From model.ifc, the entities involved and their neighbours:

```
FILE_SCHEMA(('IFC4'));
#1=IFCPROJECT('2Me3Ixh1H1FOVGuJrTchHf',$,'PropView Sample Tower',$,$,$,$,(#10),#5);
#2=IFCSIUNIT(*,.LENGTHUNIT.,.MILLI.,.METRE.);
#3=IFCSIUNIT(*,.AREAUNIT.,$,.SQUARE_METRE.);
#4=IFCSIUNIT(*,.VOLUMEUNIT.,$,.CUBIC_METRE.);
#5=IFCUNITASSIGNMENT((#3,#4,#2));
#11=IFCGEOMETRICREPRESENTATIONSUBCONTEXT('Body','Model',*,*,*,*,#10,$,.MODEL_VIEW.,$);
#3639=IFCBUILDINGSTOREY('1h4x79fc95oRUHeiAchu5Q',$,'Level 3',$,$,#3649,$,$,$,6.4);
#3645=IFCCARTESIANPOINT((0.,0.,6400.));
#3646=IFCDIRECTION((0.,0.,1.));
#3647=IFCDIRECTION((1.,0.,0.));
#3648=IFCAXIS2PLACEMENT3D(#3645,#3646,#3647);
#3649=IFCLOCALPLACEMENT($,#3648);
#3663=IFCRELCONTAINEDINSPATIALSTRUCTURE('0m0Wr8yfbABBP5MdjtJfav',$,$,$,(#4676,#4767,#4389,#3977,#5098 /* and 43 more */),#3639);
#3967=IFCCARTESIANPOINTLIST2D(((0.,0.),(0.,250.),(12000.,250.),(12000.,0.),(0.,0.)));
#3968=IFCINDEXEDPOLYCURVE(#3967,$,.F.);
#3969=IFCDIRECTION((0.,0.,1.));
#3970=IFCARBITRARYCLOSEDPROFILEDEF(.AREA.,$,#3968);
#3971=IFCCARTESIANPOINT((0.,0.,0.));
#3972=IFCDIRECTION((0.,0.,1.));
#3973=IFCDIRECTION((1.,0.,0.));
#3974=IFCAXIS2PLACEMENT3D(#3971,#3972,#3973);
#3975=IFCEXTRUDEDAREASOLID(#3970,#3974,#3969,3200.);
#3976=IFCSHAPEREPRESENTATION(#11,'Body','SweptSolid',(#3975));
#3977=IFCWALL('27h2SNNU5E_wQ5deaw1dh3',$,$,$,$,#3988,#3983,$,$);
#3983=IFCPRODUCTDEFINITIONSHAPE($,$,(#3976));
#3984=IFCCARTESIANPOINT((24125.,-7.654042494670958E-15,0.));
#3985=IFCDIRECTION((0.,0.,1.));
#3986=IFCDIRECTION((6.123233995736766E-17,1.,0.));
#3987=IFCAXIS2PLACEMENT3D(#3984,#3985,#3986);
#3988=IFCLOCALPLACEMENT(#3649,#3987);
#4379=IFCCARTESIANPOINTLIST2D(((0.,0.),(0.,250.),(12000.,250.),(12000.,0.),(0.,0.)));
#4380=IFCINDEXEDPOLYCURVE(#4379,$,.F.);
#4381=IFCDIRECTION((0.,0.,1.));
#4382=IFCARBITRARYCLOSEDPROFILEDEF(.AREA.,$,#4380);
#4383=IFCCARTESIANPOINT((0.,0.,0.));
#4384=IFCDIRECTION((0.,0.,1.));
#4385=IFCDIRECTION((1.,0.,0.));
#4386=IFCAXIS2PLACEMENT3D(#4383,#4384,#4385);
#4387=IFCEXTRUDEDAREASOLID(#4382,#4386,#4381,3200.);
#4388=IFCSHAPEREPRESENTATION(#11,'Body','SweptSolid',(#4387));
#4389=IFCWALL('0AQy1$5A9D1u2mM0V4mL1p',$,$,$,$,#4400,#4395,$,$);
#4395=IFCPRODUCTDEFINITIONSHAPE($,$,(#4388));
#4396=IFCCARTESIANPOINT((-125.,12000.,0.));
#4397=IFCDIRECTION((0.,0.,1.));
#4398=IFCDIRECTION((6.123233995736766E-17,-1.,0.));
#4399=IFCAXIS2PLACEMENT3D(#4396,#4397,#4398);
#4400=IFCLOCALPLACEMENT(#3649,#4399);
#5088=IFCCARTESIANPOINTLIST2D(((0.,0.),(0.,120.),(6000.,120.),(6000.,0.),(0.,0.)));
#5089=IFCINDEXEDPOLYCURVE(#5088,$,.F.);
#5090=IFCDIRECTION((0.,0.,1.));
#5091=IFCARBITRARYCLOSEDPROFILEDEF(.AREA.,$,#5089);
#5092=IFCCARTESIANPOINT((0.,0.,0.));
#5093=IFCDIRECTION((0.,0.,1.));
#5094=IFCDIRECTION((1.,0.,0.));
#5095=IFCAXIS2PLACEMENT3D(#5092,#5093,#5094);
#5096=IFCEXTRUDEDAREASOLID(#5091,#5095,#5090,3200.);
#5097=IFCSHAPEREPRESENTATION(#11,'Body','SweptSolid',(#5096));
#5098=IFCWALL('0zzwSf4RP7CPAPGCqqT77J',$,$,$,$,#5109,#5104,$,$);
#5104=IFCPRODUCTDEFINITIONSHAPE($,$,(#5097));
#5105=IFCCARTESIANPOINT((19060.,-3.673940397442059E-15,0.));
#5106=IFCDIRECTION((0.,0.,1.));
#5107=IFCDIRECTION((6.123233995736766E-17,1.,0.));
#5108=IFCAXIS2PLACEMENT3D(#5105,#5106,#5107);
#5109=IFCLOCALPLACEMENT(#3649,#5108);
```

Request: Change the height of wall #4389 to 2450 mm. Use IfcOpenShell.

```python
import ifcopenshell
import ifcopenshell.geom
import ifcopenshell.util.representation
import ifcopenshell.util.shape
import ifcopenshell.util.unit

model = ifcopenshell.open("model.ifc")
unit_scale = ifcopenshell.util.unit.calculate_unit_scale(model)
settings = ifcopenshell.geom.settings()


def volume(element):
    """Net volume in cubic metres, openings subtracted."""
    shape = ifcopenshell.geom.create_shape(settings, element)
    return ifcopenshell.util.shape.get_volume(shape.geometry)


wall = model.by_id(4389)
before = volume(wall)

body = ifcopenshell.util.representation.get_representation(wall, "Model", "Body")
solid = body.Items[0]
old_height = solid.Depth
solid.Depth = 2.45 / unit_scale
after = volume(wall)

print(f"height {old_height:g} -> {solid.Depth:g}, volume {before:.3f} -> {after:.3f} m3")

model.write("model-out.ifc")
```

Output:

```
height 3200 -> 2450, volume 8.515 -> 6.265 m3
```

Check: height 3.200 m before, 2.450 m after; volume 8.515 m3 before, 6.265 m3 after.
